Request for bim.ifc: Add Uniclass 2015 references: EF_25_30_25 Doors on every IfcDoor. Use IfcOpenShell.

First a look at what the model holds.

```python
import ifcopenshell

model = ifcopenshell.open("bim.ifc")
print(model.schema)
print("classifications:", [c.Name for c in model.by_type("IfcClassification")])
for ifc_class in ("IfcDoor", "IfcRoof", "IfcStair", "IfcWall", "IfcWindow"):
    print(ifc_class, len(model.by_type(ifc_class)))
```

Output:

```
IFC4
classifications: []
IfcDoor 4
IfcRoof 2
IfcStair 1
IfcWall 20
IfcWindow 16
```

```python
import ifcopenshell
import ifcopenshell.api.classification

model = ifcopenshell.open("bim.ifc")

system = ifcopenshell.api.classification.add_classification(model, classification="Uniclass 2015")

codes = {
    "IfcDoor": ("EF_25_30_25", "Doors"),
}
for ifc_class, (code, name) in codes.items():
    products = model.by_type(ifc_class)
    ifcopenshell.api.classification.add_reference(
        model, products=products, classification=system, identification=code, name=name
    )
    print(code, len(products))

model.write("bim-out.ifc")
```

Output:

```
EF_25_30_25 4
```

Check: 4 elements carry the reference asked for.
